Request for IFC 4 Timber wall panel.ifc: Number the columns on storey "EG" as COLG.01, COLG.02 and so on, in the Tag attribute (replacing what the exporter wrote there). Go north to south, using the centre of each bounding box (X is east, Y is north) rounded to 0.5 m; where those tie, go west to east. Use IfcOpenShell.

First a look at what the model holds.

```python
import ifcopenshell
import ifcopenshell.util.element
import ifcopenshell.util.placement

model = ifcopenshell.open("IFC 4 Timber wall panel.ifc")
print(model.schema)
storey = next(s for s in model.by_type("IfcBuildingStorey") if s.Name == "EG")
columns = [e for e in ifcopenshell.util.element.get_decomposition(storey) if e.is_a("IfcColumn")]
for e in sorted(columns, key=lambda e: e.id()):
    origin = ifcopenshell.util.placement.get_local_placement(e.ObjectPlacement)[:3, 3]
    print(e.id(), e.Tag, e.Name, origin.round(2) + 0.0, sep=" | ")
```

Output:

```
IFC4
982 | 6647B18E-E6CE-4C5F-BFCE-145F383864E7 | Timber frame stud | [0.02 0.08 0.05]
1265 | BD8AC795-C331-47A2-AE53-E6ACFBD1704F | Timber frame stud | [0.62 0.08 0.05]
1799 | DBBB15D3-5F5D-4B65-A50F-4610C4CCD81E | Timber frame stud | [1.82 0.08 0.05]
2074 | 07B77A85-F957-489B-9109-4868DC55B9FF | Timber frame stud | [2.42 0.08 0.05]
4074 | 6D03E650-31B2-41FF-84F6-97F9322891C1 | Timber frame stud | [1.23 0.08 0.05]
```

```python
import ifcopenshell
import ifcopenshell.geom
import ifcopenshell.util.element
import ifcopenshell.util.shape

model = ifcopenshell.open("IFC 4 Timber wall panel.ifc")
settings = ifcopenshell.geom.settings()
settings.set("use-world-coords", True)


def centre(element):
    shape = ifcopenshell.geom.create_shape(settings, element)
    return ifcopenshell.util.shape.get_bbox_centroid(shape.geometry)


storey = next(s for s in model.by_type("IfcBuildingStorey") if s.Name == "EG")
columns = [e for e in ifcopenshell.util.element.get_decomposition(storey) if e.is_a("IfcColumn")]

# Insertion points can sit at a corner or the storey origin, so sort by the geometry (in metres).
centres = {e: centre(e) for e in columns}
columns.sort(key=lambda e: (-round(centres[e][1] / 0.5), centres[e][0]))

for i, e in enumerate(columns, start=1):
    number = f"COLG.{i:02d}"
    e.Tag = number
    print(e.id(), number)

model.write("IFC 4 Timber wall panel_v2.ifc")
```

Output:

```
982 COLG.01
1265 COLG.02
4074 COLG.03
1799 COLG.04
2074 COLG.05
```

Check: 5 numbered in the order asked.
